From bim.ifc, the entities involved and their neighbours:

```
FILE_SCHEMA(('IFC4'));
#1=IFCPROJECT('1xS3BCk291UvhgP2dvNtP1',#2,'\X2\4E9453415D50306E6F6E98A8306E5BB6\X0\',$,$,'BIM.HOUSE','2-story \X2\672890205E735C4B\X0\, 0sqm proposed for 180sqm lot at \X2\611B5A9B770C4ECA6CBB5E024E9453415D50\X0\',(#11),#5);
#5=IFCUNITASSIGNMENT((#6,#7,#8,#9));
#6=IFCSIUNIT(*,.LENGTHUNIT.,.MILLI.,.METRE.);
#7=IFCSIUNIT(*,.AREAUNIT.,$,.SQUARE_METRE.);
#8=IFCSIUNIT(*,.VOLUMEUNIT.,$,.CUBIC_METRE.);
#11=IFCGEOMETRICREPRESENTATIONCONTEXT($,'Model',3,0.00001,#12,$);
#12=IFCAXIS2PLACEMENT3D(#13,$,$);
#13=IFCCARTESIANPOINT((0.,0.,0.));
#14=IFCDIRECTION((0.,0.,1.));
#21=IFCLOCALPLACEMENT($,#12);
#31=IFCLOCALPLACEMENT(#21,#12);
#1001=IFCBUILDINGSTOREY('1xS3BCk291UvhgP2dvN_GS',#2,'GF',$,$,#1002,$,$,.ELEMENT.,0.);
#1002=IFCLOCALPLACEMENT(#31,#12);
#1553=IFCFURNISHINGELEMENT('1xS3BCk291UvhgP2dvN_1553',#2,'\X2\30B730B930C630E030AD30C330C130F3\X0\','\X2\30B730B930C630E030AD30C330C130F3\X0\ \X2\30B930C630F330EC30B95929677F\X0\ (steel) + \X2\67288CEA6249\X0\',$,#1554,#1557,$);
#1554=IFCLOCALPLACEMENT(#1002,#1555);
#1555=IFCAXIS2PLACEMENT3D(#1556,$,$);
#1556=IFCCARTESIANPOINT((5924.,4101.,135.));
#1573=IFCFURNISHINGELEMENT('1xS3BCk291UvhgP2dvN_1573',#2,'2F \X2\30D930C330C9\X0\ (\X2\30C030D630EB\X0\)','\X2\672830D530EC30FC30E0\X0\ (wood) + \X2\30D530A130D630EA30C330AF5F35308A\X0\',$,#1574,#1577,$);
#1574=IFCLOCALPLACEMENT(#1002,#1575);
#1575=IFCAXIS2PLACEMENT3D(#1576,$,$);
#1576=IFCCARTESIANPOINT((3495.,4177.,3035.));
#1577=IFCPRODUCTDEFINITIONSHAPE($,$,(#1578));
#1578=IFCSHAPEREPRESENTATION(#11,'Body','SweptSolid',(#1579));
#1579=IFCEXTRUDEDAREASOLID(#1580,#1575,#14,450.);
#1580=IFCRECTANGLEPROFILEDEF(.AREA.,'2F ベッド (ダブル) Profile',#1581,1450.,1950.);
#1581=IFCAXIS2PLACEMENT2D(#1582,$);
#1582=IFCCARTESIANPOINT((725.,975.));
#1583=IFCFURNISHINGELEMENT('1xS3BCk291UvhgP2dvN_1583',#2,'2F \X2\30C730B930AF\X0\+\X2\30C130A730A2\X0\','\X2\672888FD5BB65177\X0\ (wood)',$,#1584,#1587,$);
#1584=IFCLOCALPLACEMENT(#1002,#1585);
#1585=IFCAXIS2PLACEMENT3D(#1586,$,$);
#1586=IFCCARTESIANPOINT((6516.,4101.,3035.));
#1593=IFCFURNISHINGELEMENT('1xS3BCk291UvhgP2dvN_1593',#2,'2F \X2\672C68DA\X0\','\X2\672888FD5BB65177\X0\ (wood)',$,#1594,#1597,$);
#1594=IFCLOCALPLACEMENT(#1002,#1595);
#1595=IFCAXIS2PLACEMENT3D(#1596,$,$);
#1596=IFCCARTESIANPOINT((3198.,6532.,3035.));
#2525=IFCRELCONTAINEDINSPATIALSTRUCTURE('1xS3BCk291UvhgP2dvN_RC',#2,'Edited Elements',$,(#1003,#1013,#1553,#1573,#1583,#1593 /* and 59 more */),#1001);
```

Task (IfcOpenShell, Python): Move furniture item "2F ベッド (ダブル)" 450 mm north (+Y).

```python
import ifcopenshell
import ifcopenshell.api.geometry
import ifcopenshell.util.placement

model = ifcopenshell.open("bim.ifc")

item = model.by_id(1573)
matrix = ifcopenshell.util.placement.get_local_placement(item.ObjectPlacement)
matrix[1, 3] += 450.0
ifcopenshell.api.geometry.edit_object_placement(model, product=item, matrix=matrix, is_si=False)

print(ifcopenshell.util.placement.get_local_placement(item.ObjectPlacement).round(3) + 0.0)

model.write("bim_rev.ifc")
```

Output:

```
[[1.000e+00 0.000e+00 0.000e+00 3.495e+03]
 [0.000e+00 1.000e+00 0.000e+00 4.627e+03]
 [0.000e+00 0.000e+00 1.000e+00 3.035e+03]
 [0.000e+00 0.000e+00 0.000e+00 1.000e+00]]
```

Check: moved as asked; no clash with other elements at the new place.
